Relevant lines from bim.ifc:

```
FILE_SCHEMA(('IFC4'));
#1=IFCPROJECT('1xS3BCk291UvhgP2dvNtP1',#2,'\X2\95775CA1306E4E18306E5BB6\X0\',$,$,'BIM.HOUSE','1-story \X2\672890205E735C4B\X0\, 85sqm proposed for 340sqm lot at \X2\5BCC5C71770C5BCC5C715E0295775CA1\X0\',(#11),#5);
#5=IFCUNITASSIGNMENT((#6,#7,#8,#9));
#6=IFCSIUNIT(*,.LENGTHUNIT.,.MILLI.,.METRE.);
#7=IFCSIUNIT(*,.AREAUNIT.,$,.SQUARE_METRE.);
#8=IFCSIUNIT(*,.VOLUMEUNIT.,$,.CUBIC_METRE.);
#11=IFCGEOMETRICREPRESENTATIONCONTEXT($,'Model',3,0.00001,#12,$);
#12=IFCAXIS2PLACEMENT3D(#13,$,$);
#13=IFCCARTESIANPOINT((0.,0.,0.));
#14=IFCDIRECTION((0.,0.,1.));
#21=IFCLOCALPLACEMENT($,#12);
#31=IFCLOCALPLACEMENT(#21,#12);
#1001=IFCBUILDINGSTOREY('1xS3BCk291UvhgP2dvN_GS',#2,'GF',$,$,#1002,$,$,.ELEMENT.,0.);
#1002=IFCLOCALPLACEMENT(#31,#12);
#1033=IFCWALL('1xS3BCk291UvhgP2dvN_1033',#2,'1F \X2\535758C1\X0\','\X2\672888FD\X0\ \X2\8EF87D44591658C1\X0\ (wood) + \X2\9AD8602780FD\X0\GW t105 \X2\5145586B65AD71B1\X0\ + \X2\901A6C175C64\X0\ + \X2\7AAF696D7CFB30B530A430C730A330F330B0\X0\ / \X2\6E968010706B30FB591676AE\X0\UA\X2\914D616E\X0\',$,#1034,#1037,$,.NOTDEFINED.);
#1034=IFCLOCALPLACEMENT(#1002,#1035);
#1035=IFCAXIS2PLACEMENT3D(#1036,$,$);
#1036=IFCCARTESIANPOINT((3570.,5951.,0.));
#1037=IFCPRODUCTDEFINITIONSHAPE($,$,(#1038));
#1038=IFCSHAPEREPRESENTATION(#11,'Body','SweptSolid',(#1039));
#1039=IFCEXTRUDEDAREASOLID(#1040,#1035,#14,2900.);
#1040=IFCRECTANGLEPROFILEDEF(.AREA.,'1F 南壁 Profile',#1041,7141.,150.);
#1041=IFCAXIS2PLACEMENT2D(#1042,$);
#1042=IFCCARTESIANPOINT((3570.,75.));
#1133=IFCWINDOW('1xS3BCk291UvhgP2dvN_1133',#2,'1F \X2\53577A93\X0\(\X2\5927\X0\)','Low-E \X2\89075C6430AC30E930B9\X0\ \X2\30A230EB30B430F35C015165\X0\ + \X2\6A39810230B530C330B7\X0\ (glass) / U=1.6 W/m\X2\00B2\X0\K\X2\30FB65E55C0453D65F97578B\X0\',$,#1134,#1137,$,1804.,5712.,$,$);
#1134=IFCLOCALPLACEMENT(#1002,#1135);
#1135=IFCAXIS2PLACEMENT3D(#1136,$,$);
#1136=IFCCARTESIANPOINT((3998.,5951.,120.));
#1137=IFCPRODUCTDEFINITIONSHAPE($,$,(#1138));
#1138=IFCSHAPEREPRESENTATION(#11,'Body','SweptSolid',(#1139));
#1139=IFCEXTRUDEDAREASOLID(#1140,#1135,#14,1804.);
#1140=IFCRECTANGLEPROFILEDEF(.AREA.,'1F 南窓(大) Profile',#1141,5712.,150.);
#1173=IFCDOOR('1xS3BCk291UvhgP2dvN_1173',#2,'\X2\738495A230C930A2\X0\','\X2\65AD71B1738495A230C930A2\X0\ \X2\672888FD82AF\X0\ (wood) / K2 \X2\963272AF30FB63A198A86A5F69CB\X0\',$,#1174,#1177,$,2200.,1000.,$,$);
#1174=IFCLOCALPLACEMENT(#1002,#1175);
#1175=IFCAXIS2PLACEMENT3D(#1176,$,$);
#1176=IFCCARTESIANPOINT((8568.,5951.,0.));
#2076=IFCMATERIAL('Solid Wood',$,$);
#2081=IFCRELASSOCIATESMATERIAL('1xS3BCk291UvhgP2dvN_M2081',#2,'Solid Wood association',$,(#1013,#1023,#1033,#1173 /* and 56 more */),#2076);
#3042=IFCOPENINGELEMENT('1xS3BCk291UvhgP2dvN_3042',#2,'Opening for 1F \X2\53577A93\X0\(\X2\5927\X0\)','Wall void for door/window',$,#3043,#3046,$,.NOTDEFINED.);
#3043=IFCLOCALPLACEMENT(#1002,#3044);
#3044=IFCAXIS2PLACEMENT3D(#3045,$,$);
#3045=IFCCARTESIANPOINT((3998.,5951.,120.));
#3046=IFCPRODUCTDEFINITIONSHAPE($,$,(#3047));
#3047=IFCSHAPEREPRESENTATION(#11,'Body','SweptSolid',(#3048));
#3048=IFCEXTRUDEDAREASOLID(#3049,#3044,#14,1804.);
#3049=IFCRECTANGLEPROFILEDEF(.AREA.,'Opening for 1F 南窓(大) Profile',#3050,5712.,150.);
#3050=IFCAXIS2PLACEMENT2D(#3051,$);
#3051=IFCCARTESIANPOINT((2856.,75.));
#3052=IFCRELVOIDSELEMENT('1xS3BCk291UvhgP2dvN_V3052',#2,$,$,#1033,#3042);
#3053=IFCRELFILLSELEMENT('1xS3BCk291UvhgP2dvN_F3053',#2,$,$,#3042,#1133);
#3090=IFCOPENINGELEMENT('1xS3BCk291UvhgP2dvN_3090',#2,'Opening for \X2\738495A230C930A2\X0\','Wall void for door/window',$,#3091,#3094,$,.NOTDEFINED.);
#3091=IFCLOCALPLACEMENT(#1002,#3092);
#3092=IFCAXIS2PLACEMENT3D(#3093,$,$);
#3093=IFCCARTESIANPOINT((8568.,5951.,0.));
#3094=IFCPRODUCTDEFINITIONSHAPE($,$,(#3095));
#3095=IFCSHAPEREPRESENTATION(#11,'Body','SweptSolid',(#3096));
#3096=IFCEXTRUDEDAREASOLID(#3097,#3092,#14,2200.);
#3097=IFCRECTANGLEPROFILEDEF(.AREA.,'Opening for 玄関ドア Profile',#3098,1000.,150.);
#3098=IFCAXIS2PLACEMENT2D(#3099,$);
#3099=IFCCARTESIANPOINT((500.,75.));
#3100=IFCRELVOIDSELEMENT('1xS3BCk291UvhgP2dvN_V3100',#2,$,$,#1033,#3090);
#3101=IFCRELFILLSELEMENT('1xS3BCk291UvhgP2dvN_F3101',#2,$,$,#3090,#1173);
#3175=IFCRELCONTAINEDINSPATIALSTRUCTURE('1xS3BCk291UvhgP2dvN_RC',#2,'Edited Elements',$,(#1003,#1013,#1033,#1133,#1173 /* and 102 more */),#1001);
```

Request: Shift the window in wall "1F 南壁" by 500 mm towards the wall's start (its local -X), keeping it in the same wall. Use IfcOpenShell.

```python
import ifcopenshell
import ifcopenshell.api.geometry
import ifcopenshell.util.placement
import ifcopenshell.util.unit

model = ifcopenshell.open("bim.ifc")
unit_scale = ifcopenshell.util.unit.calculate_unit_scale(model)

window = model.by_guid("1xS3BCk291UvhgP2dvN_1133")
opening = window.FillsVoids[0].RelatingOpeningElement
wall = opening.VoidsElements[0].RelatingBuildingElement

wall_matrix = ifcopenshell.util.placement.get_local_placement(wall.ObjectPlacement)
shift = wall_matrix[:3, 0] * -0.5 / unit_scale
before = ifcopenshell.util.placement.get_local_placement(window.ObjectPlacement)[:3, 3].copy()

# The window is not placed relative to its opening, so move both.
for product in (opening, window):
    matrix = ifcopenshell.util.placement.get_local_placement(product.ObjectPlacement)
    matrix[:3, 3] += shift
    ifcopenshell.api.geometry.edit_object_placement(model, product=product, matrix=matrix, is_si=False)

after = ifcopenshell.util.placement.get_local_placement(window.ObjectPlacement)[:3, 3]
print("window moved by", (after - before).round(3) + 0.0)

model.write("bim_v2.ifc")
```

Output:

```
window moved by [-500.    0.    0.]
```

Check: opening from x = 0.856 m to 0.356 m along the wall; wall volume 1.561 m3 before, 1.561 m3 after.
